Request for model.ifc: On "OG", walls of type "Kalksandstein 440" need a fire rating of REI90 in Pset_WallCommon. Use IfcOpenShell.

First a look at what the model holds.

```python
import ifcopenshell
import ifcopenshell.util.element

model = ifcopenshell.open("model.ifc")
print(model.schema)
storey = next(s for s in model.by_type("IfcBuildingStorey") if s.Name == "OG")
walls = [e for e in ifcopenshell.util.element.get_decomposition(storey) if e.is_a("IfcWall")]
seen = {}
for e in walls:
    element_type = ifcopenshell.util.element.get_type(e)
    key = (element_type.Name if element_type != e and element_type else None, ifcopenshell.util.element.get_pset(e, "Pset_WallCommon", "FireRating"))
    seen[key] = seen.get(key, 0) + 1
for (name, value), count in sorted(seen.items(), key=str):
    print(count, "x", name, "|", value)
```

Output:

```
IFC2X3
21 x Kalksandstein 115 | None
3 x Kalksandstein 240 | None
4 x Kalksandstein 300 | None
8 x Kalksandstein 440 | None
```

```python
import ifcopenshell
import ifcopenshell.api.pset
import ifcopenshell.util.element

model = ifcopenshell.open("model.ifc")

storey = next(s for s in model.by_type("IfcBuildingStorey") if s.Name == "OG")
walls = [e for e in ifcopenshell.util.element.get_decomposition(storey) if e.is_a("IfcWall")]

count = 0
for e in walls:
    element_type = ifcopenshell.util.element.get_type(e)
    if element_type in (None, e) or element_type.Name != "Kalksandstein 440":
        continue
    # add_pset returns the element's existing set when there is one.
    pset = ifcopenshell.api.pset.add_pset(model, product=e, name="Pset_WallCommon")
    ifcopenshell.api.pset.edit_pset(model, pset=pset, properties={"FireRating": "REI90"})
    count += 1

print(count, "walls updated")

model.write("model_edited.ifc")
```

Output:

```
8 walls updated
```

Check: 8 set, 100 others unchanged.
